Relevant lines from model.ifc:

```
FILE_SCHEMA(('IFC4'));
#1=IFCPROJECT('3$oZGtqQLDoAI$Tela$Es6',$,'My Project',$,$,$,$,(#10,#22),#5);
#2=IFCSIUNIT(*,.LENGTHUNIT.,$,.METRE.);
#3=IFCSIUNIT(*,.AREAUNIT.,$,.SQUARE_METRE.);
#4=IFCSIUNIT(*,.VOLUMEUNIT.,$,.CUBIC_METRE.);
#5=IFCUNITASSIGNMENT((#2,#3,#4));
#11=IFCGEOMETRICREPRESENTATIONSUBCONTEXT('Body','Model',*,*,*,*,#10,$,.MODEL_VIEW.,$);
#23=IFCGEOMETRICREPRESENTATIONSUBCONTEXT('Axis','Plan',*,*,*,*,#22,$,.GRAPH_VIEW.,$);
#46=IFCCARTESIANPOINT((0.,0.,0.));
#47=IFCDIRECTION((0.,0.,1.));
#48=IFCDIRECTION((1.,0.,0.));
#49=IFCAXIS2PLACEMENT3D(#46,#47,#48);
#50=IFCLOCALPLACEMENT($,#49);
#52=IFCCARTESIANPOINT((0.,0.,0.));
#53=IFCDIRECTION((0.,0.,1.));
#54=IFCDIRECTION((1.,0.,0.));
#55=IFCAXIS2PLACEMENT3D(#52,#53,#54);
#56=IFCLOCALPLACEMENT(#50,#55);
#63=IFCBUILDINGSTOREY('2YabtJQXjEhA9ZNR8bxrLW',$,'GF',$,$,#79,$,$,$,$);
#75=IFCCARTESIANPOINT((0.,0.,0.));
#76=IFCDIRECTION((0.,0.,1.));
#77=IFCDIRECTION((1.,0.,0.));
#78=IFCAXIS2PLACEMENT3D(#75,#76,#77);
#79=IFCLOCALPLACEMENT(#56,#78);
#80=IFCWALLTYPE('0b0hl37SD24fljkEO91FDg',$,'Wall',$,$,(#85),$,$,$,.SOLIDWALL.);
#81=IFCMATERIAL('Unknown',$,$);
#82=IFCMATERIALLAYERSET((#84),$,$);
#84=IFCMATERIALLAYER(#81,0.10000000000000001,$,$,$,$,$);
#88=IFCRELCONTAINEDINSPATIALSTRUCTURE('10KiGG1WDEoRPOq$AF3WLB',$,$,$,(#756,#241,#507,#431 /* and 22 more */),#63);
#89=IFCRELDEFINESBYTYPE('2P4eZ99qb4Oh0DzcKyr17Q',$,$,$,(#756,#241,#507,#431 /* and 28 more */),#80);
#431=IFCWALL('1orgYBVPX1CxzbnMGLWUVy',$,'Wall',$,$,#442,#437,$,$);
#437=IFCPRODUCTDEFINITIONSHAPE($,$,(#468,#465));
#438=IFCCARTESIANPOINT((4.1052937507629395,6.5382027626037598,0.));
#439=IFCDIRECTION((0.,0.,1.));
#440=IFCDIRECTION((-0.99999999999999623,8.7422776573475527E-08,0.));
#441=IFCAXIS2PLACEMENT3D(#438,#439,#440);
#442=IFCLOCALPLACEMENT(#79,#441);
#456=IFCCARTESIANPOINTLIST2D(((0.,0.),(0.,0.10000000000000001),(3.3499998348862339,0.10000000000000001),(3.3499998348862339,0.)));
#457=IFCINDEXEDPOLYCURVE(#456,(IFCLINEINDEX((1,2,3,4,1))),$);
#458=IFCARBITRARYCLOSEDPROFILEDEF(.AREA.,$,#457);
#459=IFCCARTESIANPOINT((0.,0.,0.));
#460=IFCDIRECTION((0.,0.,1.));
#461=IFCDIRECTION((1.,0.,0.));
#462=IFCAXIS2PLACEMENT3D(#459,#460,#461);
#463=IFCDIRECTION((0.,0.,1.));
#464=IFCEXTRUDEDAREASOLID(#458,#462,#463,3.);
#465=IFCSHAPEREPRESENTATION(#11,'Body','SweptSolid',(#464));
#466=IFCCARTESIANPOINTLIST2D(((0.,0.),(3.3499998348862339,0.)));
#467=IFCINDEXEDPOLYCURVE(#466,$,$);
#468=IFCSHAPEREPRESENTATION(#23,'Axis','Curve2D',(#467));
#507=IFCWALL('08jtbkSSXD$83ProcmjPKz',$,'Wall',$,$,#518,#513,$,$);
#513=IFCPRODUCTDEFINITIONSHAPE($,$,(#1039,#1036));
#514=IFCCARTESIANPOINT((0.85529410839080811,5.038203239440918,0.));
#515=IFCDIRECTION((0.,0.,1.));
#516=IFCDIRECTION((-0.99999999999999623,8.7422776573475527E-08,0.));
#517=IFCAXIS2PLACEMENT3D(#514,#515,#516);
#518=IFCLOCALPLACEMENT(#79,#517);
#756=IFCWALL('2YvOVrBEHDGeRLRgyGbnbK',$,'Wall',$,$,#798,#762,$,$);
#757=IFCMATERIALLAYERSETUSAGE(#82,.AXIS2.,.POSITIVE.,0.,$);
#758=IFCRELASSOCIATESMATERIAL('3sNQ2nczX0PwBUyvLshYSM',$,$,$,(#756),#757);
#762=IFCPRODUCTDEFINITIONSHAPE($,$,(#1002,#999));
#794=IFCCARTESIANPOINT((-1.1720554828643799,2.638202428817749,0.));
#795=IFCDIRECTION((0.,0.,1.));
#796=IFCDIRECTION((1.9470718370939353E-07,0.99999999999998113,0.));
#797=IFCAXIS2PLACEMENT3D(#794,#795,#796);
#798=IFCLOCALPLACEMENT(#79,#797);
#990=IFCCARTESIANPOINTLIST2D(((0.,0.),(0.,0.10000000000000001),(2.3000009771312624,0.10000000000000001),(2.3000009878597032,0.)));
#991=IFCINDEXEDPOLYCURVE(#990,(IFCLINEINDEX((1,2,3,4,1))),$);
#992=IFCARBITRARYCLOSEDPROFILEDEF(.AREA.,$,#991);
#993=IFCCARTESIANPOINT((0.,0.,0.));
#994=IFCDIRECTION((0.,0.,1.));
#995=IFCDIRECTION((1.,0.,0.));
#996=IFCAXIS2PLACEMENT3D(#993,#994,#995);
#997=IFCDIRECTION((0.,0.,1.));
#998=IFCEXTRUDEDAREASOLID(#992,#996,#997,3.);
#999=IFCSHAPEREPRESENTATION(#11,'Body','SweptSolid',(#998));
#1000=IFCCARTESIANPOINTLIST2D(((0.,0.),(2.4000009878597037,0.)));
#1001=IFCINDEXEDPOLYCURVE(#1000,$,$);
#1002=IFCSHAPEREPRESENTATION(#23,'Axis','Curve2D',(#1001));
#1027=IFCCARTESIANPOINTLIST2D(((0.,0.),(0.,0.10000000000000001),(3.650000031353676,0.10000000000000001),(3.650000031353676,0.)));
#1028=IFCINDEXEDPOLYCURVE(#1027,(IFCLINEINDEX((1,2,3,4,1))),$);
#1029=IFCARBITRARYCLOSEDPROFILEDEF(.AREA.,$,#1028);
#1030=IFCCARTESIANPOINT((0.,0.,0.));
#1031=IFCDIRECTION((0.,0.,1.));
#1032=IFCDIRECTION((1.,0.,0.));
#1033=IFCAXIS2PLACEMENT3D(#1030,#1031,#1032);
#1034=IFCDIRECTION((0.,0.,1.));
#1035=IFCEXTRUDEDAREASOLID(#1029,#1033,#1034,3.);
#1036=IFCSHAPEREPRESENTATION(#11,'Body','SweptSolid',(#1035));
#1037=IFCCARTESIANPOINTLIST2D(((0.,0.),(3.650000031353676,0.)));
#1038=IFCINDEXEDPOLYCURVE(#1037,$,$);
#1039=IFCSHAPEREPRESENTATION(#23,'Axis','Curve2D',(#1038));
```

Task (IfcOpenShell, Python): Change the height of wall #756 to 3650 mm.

```python
import ifcopenshell
import ifcopenshell.geom
import ifcopenshell.util.representation
import ifcopenshell.util.shape
import ifcopenshell.util.unit

model = ifcopenshell.open("model.ifc")
unit_scale = ifcopenshell.util.unit.calculate_unit_scale(model)
settings = ifcopenshell.geom.settings()


def volume(element):
    """Net volume in cubic metres, openings subtracted."""
    shape = ifcopenshell.geom.create_shape(settings, element)
    return ifcopenshell.util.shape.get_volume(shape.geometry)


wall = model.by_id(756)
before = volume(wall)

body = ifcopenshell.util.representation.get_representation(wall, "Model", "Body")
solid = body.Items[0]
old_height = solid.Depth
solid.Depth = 3.65 / unit_scale
after = volume(wall)

print(f"height {old_height:g} -> {solid.Depth:g}, volume {before:.3f} -> {after:.3f} m3")

model.write("model_updated.ifc")
```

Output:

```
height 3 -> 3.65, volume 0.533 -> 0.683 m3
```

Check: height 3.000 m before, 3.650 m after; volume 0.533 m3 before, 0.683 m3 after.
